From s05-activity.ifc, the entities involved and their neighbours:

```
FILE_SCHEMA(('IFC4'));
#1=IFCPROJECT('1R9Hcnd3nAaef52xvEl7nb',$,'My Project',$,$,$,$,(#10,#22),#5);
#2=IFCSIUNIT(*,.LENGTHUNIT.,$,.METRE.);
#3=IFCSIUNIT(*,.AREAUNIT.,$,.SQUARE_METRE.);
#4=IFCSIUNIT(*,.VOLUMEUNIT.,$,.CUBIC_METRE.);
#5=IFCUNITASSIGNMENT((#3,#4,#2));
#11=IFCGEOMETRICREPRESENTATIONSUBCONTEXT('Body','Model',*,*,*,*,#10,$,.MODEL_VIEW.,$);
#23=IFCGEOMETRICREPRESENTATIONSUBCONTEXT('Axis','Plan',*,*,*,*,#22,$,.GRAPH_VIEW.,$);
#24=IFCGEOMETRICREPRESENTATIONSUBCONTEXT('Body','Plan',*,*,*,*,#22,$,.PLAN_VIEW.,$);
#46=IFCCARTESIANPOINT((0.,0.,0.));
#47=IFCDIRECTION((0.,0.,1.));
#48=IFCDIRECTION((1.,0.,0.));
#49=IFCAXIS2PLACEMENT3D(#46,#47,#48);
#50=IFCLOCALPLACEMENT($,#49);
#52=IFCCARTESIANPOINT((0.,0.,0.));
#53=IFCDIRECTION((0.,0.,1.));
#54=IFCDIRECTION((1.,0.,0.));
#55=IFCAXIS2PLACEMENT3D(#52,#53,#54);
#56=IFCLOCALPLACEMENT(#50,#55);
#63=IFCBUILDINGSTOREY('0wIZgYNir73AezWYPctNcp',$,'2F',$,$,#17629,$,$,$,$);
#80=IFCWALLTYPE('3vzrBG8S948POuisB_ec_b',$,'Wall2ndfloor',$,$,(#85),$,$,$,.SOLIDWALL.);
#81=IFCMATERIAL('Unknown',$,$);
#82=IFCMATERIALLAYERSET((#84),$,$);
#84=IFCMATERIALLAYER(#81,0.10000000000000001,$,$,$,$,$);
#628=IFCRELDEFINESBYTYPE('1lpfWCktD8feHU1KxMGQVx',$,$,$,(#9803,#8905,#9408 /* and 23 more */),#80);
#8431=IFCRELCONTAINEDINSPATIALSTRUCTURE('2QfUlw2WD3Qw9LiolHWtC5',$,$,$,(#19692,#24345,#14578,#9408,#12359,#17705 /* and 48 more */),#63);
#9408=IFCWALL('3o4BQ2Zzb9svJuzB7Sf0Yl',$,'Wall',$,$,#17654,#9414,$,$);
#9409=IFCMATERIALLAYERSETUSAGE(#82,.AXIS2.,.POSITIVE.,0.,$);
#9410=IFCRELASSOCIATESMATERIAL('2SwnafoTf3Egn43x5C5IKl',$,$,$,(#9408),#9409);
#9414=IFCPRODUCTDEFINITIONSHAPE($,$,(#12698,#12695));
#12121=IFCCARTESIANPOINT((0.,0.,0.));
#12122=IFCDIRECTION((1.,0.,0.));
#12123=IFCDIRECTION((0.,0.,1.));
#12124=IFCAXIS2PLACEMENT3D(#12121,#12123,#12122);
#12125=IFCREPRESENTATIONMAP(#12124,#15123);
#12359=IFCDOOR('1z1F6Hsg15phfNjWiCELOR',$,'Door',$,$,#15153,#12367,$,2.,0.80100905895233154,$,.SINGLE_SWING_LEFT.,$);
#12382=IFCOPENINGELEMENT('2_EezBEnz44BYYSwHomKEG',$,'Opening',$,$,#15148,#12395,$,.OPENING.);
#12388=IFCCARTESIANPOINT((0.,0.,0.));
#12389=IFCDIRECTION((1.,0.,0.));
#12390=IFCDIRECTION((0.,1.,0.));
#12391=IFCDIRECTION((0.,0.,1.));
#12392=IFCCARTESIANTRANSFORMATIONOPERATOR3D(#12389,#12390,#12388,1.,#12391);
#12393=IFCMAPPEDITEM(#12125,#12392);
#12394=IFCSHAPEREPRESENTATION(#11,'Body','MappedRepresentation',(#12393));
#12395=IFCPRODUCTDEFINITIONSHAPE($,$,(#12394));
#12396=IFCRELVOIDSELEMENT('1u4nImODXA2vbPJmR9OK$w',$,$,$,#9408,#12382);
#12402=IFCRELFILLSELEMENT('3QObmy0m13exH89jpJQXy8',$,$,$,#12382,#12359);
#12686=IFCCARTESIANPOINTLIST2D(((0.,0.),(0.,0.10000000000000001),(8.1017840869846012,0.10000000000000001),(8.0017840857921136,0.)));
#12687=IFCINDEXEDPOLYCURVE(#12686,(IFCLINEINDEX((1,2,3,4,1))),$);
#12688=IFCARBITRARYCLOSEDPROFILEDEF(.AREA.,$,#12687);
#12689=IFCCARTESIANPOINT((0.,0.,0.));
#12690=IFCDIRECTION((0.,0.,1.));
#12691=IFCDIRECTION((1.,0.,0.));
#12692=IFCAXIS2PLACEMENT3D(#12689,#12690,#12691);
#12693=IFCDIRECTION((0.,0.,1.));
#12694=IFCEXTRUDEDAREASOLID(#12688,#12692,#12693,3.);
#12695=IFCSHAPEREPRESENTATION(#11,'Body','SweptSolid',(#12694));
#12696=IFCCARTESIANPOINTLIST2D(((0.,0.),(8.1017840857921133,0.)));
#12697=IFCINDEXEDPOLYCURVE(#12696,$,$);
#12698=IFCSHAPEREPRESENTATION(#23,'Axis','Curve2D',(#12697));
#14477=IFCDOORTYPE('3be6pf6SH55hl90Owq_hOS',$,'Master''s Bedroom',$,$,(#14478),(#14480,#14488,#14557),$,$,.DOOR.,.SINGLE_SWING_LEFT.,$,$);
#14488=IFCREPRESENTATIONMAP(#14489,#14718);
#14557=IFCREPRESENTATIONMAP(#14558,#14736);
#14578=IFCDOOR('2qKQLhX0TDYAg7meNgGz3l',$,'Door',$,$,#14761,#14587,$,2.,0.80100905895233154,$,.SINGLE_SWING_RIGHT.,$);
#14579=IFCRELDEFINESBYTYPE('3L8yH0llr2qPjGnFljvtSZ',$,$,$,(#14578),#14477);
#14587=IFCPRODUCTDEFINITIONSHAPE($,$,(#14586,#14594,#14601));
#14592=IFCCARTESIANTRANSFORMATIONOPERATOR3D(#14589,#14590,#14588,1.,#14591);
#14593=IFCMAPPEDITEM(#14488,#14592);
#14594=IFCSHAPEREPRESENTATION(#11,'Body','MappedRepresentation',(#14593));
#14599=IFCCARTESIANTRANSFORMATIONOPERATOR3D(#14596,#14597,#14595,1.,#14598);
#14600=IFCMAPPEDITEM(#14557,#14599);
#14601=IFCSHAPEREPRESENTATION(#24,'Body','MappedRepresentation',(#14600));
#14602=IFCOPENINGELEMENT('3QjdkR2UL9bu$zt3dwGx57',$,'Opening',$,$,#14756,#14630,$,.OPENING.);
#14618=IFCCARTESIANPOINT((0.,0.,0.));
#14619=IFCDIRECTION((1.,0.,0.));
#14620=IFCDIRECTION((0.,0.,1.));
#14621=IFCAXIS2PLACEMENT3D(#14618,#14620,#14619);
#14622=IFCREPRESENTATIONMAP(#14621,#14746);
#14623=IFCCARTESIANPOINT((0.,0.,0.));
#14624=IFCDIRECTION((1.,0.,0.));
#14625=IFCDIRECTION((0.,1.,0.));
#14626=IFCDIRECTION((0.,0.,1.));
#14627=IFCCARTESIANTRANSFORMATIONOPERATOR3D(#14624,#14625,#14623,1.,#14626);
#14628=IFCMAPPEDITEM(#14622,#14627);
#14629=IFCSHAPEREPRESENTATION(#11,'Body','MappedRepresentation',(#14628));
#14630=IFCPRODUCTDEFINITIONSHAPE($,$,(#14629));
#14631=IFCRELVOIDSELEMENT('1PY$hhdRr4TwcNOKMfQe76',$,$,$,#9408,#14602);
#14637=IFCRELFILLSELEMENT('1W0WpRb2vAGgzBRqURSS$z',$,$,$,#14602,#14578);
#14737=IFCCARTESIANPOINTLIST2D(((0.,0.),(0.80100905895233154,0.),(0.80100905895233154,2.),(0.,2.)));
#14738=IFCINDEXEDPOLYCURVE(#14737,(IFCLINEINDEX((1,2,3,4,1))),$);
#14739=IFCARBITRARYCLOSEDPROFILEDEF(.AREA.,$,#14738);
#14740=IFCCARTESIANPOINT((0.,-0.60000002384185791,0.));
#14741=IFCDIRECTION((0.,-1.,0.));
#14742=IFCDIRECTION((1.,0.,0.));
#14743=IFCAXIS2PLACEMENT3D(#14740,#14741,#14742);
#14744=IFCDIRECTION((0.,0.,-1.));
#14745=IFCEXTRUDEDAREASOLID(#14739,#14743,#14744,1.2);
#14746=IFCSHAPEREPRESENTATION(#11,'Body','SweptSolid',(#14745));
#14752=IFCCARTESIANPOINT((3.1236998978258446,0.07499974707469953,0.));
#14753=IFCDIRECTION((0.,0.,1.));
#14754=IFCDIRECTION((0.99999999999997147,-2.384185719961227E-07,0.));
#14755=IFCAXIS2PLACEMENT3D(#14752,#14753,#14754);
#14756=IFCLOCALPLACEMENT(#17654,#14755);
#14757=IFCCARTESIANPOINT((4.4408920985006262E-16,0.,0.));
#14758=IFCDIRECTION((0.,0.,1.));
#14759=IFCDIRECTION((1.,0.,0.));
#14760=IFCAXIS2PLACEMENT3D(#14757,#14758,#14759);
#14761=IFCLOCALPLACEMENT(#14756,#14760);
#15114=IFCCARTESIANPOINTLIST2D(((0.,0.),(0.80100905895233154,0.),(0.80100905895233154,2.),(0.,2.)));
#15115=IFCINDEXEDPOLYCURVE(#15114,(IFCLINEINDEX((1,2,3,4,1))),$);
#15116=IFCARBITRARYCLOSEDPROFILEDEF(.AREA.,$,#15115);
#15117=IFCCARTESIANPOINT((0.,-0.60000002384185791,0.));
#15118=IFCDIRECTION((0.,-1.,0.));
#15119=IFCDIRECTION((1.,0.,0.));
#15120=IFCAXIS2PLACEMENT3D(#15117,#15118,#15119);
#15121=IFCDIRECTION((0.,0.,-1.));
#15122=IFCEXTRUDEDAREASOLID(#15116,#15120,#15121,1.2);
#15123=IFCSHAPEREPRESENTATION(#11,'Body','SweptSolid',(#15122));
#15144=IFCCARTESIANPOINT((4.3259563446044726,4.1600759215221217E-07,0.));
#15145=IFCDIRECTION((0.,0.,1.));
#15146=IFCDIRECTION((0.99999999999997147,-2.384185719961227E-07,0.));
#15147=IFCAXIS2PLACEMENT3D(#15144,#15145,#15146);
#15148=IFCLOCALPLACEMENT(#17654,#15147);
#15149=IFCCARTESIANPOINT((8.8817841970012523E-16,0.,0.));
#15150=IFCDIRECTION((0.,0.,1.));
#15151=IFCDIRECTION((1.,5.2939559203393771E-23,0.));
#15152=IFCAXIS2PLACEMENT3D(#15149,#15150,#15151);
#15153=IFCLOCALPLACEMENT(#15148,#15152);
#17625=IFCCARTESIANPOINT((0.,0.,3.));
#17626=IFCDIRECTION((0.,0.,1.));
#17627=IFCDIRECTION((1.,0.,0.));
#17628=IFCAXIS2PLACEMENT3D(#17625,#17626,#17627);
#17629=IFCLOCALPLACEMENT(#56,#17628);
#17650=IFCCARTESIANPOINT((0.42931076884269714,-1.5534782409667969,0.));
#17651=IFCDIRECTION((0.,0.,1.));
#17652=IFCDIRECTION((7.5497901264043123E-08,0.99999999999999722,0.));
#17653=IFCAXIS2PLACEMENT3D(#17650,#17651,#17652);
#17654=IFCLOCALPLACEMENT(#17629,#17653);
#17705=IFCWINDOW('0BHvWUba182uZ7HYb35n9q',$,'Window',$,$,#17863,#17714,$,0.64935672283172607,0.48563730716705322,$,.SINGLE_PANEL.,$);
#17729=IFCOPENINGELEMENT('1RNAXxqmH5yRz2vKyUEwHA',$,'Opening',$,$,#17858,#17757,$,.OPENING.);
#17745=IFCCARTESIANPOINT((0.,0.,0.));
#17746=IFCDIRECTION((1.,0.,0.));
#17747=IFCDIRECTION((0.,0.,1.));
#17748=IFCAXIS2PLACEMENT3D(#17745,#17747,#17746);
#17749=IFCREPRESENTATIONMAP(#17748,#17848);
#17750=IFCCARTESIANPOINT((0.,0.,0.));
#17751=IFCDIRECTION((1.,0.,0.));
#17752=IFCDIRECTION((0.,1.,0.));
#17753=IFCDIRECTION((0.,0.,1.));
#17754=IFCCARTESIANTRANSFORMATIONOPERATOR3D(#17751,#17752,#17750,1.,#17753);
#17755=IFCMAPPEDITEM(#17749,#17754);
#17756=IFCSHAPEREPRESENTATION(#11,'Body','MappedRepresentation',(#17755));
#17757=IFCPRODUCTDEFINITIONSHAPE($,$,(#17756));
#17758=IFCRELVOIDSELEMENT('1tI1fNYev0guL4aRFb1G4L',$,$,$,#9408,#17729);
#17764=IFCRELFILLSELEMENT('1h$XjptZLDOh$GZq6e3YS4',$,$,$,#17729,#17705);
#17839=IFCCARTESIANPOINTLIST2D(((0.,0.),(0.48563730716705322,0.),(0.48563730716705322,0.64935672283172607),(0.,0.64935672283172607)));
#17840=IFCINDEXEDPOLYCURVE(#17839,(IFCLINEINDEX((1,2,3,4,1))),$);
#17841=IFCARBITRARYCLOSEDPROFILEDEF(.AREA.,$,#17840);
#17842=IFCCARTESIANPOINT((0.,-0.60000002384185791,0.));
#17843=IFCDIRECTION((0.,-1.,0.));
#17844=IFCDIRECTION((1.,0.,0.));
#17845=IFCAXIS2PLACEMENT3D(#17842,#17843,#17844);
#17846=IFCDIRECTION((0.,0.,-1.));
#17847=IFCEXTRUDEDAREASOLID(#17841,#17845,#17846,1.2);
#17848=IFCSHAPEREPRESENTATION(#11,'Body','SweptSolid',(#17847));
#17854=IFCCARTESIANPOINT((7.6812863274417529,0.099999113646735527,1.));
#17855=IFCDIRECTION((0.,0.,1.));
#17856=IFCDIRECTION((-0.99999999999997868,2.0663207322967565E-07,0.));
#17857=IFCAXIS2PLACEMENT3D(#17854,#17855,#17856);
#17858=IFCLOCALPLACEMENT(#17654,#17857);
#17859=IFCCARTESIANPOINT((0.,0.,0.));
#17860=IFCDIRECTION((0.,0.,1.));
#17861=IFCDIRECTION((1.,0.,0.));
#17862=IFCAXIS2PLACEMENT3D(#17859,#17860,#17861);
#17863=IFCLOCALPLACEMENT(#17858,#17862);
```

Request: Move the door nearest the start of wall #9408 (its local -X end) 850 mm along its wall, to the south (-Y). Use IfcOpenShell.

```python
import ifcopenshell
import ifcopenshell.api.geometry
import ifcopenshell.util.placement

model = ifcopenshell.open("s05-activity.ifc")

door = model.by_guid("2qKQLhX0TDYAg7meNgGz3l")
opening = door.FillsVoids[0].RelatingOpeningElement
wall = opening.VoidsElements[0].RelatingBuildingElement

wall_matrix = ifcopenshell.util.placement.get_local_placement(wall.ObjectPlacement)
shift = wall_matrix[:3, 0] * -0.85
before = ifcopenshell.util.placement.get_local_placement(door.ObjectPlacement)[:3, 3].copy()

# The door is placed relative to its opening, so it follows when the opening moves.
matrix = ifcopenshell.util.placement.get_local_placement(opening.ObjectPlacement)
matrix[:3, 3] += shift
ifcopenshell.api.geometry.edit_object_placement(
    model, product=opening, matrix=matrix, is_si=False, should_transform_children=True
)

after = ifcopenshell.util.placement.get_local_placement(door.ObjectPlacement)[:3, 3]
print("door moved by", (after - before).round(3) + 0.0)

model.write("s05-activity_edited.ifc")
```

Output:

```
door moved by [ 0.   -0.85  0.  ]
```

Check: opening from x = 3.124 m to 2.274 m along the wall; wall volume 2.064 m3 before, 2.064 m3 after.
